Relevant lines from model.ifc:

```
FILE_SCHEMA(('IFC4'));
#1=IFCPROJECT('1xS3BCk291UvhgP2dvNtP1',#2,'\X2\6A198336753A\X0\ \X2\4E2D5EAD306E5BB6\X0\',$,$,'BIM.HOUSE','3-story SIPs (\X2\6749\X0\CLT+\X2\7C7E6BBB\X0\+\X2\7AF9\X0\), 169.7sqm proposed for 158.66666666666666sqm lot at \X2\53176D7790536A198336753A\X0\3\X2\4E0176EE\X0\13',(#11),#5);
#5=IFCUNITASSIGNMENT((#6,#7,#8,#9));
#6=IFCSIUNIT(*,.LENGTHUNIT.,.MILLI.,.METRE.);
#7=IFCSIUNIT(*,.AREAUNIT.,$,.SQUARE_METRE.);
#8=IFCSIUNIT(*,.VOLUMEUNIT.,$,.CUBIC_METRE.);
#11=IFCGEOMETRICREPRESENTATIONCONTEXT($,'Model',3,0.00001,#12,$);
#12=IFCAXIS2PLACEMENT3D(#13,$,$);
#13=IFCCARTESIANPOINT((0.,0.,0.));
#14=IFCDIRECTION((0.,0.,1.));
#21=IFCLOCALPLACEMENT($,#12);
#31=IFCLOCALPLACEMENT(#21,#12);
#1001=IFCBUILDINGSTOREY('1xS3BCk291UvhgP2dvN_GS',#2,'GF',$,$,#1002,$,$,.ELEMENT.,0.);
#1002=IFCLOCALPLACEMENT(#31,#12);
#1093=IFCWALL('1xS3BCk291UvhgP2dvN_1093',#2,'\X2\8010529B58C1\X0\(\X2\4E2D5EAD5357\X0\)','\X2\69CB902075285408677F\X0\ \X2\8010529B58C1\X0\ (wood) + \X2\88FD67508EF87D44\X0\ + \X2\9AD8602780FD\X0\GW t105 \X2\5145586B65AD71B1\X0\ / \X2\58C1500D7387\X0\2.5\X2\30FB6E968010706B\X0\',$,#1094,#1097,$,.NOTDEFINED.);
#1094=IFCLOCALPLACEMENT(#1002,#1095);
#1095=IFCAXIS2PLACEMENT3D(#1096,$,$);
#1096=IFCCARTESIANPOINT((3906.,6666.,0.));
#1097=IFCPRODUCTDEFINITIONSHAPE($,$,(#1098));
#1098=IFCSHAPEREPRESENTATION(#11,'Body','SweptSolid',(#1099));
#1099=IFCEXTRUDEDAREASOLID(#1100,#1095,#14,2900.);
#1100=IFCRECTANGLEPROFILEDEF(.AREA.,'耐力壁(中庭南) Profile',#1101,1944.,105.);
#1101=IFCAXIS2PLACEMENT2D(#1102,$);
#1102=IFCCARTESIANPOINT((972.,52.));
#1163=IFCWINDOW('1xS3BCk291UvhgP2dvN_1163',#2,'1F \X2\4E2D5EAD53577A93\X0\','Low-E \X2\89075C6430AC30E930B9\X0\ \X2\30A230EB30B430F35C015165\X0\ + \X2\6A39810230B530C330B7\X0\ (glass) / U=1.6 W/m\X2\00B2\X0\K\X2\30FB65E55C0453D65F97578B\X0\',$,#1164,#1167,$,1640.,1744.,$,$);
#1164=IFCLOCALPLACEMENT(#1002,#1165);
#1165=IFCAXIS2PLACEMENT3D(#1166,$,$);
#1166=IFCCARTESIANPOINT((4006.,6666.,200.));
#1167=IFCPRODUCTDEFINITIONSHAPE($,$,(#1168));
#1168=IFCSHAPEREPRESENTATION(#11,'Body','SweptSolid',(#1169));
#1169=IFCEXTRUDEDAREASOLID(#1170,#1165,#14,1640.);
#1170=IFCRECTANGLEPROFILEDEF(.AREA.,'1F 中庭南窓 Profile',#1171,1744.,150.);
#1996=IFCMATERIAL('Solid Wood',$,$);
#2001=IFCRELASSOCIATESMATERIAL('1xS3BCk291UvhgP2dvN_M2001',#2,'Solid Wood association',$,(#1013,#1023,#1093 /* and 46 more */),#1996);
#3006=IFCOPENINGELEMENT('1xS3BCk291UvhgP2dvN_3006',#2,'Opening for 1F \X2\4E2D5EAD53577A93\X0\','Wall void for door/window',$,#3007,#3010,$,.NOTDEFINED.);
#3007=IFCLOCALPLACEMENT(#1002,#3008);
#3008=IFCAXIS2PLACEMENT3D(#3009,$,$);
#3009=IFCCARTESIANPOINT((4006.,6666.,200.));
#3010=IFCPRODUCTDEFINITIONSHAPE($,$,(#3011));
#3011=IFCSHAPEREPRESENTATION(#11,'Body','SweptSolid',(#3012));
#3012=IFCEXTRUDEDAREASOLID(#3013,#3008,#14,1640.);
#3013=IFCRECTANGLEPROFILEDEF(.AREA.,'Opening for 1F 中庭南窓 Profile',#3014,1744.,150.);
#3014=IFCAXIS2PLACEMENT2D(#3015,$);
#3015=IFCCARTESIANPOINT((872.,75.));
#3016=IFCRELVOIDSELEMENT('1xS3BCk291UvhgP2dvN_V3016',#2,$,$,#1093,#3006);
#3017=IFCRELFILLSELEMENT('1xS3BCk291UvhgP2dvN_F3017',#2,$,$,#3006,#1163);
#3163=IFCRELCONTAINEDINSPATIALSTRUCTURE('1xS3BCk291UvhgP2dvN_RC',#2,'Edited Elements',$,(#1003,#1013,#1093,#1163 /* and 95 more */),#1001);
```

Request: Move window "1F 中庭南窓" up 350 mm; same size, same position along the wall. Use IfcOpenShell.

```python
import numpy as np
import ifcopenshell
import ifcopenshell.api.geometry
import ifcopenshell.util.placement
import ifcopenshell.util.unit

model = ifcopenshell.open("model.ifc")
unit_scale = ifcopenshell.util.unit.calculate_unit_scale(model)

window = model.by_id(1163)
opening = window.FillsVoids[0].RelatingOpeningElement
dz = 0.35 / unit_scale

shift = np.array([0.0, 0.0, dz])
# The window is not placed relative to its opening, so move both.
for product in (opening, window):
    matrix = ifcopenshell.util.placement.get_local_placement(product.ObjectPlacement)
    matrix[:3, 3] += shift
    ifcopenshell.api.geometry.edit_object_placement(model, product=product, matrix=matrix, is_si=False)

print(f"moved by {dz * unit_scale:+.3f} m")

model.write("model_v2.ifc")
```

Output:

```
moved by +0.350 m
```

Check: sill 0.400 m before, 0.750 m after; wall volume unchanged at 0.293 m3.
